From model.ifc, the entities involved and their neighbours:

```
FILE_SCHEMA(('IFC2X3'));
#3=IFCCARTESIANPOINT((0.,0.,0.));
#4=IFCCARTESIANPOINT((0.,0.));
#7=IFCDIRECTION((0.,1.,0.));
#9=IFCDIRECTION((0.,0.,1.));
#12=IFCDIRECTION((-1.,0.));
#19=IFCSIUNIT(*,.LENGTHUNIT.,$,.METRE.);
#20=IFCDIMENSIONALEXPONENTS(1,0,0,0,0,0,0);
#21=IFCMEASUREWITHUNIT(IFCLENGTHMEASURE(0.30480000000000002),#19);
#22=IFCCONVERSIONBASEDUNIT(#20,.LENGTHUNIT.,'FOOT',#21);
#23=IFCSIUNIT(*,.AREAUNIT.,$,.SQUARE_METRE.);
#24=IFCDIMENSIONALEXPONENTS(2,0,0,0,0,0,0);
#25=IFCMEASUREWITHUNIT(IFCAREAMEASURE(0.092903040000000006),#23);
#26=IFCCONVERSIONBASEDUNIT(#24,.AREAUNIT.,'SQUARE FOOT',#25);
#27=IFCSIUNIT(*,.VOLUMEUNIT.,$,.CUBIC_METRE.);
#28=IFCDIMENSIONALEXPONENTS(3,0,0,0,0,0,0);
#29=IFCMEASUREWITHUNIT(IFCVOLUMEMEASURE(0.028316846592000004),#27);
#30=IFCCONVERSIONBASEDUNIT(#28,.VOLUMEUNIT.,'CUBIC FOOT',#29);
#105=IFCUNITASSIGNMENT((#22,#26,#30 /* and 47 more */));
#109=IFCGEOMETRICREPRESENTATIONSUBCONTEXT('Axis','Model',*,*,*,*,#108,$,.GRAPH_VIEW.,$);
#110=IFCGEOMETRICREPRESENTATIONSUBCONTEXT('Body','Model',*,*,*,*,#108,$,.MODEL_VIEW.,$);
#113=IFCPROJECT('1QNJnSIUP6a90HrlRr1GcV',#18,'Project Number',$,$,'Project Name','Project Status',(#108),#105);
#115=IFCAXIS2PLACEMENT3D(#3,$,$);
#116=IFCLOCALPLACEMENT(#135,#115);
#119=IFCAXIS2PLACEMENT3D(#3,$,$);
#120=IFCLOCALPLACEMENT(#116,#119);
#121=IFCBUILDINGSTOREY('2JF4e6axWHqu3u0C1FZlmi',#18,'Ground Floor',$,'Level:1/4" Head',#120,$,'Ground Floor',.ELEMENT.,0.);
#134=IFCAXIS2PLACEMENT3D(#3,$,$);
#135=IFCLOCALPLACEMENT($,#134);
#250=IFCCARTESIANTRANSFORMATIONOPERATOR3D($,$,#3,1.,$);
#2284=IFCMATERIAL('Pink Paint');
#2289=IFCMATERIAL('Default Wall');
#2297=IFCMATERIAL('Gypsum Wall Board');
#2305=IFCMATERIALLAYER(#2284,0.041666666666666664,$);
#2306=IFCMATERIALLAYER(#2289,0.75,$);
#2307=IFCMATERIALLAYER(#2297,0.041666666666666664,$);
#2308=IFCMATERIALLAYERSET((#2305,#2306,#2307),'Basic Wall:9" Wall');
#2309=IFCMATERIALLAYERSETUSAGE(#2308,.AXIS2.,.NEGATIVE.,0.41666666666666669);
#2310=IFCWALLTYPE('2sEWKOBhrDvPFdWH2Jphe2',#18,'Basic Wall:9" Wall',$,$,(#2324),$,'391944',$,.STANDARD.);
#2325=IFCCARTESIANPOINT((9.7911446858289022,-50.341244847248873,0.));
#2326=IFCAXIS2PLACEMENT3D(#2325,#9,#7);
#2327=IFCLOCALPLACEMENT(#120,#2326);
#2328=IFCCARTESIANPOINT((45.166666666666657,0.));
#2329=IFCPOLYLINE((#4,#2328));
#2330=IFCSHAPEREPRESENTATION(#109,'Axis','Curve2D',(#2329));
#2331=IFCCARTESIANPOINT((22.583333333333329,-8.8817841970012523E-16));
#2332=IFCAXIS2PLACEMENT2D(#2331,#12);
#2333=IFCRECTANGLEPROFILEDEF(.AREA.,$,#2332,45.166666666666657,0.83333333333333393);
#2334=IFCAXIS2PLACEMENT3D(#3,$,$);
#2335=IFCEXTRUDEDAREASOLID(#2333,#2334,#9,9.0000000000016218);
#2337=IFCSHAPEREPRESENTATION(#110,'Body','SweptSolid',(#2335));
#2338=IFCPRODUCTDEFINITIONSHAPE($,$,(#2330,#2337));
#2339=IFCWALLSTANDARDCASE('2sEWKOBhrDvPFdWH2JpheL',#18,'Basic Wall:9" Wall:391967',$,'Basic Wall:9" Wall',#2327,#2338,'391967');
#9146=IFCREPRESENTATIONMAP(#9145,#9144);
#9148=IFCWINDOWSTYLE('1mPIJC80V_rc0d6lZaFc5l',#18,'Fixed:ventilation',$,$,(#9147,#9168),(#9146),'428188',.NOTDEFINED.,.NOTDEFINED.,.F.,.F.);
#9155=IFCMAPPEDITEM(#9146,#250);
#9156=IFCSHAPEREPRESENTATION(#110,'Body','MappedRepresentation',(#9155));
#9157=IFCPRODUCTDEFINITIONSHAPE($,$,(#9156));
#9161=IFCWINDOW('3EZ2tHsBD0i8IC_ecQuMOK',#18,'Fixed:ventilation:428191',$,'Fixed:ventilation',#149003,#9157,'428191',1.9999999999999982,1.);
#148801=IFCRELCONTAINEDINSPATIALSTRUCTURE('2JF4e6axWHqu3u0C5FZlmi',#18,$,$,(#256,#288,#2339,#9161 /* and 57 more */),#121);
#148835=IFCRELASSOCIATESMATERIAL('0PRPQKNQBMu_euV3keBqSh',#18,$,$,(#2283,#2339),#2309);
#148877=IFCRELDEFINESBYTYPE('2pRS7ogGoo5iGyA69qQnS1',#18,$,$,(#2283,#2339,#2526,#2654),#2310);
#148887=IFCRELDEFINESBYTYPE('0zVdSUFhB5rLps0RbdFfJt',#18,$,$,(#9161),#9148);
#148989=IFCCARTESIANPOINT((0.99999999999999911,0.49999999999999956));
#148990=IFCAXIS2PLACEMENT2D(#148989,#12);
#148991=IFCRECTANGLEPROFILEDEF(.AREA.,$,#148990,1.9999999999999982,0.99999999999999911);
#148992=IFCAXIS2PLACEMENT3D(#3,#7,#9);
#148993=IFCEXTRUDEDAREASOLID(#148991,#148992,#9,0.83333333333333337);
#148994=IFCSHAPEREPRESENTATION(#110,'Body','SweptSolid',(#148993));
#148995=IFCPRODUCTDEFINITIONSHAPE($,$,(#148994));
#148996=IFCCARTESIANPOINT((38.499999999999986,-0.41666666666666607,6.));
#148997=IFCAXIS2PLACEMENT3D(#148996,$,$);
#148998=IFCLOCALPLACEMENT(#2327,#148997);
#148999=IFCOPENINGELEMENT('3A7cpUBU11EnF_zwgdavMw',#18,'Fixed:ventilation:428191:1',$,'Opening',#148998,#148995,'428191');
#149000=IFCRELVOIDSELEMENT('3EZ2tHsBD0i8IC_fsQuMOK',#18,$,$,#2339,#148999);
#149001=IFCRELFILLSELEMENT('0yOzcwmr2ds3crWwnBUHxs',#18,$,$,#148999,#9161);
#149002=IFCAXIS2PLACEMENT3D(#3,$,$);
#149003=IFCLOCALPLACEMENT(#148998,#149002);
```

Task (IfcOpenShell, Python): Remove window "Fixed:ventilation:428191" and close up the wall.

```python
import ifcopenshell
import ifcopenshell.api.feature
import ifcopenshell.api.root
import ifcopenshell.geom
import ifcopenshell.util.shape

model = ifcopenshell.open("model.ifc")
settings = ifcopenshell.geom.settings()


def volume(element):
    """Net volume in cubic metres, openings subtracted."""
    shape = ifcopenshell.geom.create_shape(settings, element)
    return ifcopenshell.util.shape.get_volume(shape.geometry)


window = model.by_guid("3EZ2tHsBD0i8IC_ecQuMOK")
opening = window.FillsVoids[0].RelatingOpeningElement
wall = opening.VoidsElements[0].RelatingBuildingElement
before = volume(wall)

ifcopenshell.api.root.remove_product(model, product=window)
ifcopenshell.api.feature.remove_feature(model, feature=opening)

after = volume(wall)

print(f"wall volume {before:.3f} -> {after:.3f} m3")

model.write("model_updated.ifc")
```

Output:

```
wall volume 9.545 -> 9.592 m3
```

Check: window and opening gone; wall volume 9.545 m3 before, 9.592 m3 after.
